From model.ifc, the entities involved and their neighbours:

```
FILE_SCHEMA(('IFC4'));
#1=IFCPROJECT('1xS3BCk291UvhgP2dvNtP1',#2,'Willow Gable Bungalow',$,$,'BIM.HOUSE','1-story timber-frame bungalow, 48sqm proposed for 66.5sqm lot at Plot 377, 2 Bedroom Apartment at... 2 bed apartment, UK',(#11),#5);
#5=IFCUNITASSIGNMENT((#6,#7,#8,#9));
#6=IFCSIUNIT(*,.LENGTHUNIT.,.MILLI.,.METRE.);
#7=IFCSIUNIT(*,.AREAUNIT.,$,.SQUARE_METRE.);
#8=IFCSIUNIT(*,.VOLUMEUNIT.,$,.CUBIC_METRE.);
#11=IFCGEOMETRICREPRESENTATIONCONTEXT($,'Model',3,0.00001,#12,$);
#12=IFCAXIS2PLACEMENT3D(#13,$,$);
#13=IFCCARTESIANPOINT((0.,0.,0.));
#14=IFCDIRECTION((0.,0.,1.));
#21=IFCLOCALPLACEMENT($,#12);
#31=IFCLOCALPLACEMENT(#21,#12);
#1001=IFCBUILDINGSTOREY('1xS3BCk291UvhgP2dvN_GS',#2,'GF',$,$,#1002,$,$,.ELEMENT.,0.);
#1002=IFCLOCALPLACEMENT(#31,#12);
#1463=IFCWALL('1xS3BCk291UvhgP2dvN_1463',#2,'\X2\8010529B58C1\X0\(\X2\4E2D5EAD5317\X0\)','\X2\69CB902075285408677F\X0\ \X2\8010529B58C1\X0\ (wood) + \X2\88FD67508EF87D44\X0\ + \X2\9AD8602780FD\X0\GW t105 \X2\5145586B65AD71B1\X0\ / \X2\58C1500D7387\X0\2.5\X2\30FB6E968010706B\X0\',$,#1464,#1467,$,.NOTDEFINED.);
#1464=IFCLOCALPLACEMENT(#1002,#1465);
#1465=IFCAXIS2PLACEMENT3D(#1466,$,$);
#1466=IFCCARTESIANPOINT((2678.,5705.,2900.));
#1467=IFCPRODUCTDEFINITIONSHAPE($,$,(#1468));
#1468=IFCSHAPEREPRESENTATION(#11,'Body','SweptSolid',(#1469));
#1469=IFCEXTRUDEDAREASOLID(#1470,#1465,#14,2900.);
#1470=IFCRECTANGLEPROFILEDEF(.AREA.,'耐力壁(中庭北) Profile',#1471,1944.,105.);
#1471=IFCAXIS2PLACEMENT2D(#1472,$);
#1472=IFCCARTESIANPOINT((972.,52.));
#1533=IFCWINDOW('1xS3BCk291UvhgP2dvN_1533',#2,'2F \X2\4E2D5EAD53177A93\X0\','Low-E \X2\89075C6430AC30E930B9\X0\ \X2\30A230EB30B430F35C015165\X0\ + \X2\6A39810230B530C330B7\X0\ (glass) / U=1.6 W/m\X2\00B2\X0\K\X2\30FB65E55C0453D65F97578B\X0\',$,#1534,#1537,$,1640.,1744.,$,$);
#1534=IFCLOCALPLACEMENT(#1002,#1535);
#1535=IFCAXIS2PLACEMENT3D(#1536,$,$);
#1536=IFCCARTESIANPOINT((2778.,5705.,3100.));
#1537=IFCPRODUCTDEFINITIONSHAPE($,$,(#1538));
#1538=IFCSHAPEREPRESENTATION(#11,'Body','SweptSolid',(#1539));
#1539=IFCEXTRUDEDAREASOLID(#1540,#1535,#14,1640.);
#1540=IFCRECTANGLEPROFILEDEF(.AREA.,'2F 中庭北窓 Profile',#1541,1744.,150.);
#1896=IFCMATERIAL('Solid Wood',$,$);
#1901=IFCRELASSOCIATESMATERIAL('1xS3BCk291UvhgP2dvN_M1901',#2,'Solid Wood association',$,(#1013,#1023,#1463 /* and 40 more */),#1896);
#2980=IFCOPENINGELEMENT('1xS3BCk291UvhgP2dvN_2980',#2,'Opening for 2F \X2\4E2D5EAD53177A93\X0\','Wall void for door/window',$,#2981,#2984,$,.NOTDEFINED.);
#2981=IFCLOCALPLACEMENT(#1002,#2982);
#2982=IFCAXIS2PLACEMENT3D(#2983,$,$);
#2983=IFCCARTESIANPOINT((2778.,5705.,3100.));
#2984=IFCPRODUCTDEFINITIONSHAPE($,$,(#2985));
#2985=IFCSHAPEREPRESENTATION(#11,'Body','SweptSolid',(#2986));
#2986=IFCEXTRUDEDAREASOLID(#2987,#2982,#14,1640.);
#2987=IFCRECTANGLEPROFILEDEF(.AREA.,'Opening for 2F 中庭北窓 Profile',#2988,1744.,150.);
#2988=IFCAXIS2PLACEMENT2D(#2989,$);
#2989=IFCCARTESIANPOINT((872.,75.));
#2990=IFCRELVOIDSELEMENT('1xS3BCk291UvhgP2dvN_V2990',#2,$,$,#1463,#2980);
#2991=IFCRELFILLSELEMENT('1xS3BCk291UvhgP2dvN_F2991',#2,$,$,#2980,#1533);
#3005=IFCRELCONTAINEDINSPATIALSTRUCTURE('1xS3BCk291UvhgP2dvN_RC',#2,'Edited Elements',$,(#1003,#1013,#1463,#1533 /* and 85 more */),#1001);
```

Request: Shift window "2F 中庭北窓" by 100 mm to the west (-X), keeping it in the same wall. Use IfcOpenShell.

```python
import ifcopenshell
import ifcopenshell.api.geometry
import ifcopenshell.util.placement
import ifcopenshell.util.unit

model = ifcopenshell.open("model.ifc")
unit_scale = ifcopenshell.util.unit.calculate_unit_scale(model)

window = model.by_guid("1xS3BCk291UvhgP2dvN_1533")
opening = window.FillsVoids[0].RelatingOpeningElement
wall = opening.VoidsElements[0].RelatingBuildingElement

wall_matrix = ifcopenshell.util.placement.get_local_placement(wall.ObjectPlacement)
shift = wall_matrix[:3, 0] * -0.1 / unit_scale
before = ifcopenshell.util.placement.get_local_placement(window.ObjectPlacement)[:3, 3].copy()

# The window is not placed relative to its opening, so move both.
for product in (opening, window):
    matrix = ifcopenshell.util.placement.get_local_placement(product.ObjectPlacement)
    matrix[:3, 3] += shift
    ifcopenshell.api.geometry.edit_object_placement(model, product=product, matrix=matrix, is_si=False)

after = ifcopenshell.util.placement.get_local_placement(window.ObjectPlacement)[:3, 3]
print("window moved by", (after - before).round(3) + 0.0)

model.write("model_updated.ifc")
```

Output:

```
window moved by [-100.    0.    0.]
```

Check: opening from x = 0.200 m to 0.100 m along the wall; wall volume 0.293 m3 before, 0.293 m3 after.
